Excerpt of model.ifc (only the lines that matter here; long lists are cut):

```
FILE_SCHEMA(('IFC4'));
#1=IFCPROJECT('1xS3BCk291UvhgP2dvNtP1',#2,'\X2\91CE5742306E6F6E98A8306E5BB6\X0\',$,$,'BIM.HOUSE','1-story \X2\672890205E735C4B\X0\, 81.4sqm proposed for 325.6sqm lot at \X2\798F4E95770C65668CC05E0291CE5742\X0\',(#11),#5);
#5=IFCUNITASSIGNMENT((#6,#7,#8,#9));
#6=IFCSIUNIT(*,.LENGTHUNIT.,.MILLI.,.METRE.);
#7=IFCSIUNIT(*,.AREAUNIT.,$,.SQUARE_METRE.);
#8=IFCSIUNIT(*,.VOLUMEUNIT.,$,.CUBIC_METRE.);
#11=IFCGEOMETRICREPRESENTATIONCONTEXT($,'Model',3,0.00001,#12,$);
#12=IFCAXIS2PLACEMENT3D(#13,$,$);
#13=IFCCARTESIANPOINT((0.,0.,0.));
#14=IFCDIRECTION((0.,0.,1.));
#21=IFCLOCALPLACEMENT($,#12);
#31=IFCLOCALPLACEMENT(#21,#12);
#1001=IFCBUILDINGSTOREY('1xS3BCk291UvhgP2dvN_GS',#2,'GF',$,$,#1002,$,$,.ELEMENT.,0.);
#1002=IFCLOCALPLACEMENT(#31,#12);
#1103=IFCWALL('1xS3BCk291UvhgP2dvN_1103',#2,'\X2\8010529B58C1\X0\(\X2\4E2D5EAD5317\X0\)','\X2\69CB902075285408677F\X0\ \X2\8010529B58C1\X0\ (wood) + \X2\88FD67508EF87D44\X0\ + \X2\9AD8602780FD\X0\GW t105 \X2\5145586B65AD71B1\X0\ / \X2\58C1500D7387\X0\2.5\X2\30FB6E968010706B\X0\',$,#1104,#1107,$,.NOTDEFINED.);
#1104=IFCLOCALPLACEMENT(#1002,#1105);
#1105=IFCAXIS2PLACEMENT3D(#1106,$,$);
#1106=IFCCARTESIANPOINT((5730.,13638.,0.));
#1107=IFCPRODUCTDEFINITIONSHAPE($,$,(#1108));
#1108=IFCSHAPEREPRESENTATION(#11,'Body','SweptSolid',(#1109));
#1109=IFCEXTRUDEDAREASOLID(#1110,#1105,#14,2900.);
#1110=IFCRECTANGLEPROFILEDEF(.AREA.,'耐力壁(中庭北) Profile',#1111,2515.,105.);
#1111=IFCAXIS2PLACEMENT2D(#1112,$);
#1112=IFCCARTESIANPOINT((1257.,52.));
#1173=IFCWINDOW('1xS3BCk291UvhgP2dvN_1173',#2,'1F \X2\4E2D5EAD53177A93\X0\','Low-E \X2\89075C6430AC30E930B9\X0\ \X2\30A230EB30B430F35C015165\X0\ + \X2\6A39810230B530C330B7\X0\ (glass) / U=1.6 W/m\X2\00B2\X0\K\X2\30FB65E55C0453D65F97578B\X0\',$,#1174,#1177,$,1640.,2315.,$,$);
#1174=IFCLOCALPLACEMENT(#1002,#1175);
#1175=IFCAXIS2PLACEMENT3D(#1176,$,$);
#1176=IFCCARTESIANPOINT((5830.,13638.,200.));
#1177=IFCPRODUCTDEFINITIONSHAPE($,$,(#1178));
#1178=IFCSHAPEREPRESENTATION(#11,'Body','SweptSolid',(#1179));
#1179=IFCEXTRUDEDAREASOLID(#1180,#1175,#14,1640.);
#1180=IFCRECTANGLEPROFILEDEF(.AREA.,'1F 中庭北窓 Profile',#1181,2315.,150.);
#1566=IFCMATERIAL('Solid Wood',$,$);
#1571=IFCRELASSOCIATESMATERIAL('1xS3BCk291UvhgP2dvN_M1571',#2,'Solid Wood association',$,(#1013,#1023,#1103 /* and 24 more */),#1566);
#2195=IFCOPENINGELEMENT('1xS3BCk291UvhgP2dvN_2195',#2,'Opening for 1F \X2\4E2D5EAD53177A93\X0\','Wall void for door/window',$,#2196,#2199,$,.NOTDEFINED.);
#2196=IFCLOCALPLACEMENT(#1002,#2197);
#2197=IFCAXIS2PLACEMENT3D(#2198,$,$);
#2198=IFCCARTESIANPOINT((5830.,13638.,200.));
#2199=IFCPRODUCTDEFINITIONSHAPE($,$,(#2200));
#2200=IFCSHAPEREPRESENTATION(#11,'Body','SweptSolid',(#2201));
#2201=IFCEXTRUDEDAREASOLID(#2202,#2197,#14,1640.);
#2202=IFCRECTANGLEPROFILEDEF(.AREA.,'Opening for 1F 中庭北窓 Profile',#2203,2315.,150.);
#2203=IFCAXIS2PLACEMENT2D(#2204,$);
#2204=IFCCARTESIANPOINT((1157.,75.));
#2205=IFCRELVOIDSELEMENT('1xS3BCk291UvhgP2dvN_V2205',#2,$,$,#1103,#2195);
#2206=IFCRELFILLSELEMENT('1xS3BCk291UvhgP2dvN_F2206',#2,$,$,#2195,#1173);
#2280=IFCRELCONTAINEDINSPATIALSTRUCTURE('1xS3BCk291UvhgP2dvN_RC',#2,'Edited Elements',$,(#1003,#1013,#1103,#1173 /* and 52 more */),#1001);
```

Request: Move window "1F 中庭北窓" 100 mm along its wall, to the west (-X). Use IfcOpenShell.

```python
import ifcopenshell
import ifcopenshell.api.geometry
import ifcopenshell.util.placement
import ifcopenshell.util.unit

model = ifcopenshell.open("model.ifc")
unit_scale = ifcopenshell.util.unit.calculate_unit_scale(model)

window = model.by_guid("1xS3BCk291UvhgP2dvN_1173")
opening = window.FillsVoids[0].RelatingOpeningElement
wall = opening.VoidsElements[0].RelatingBuildingElement

wall_matrix = ifcopenshell.util.placement.get_local_placement(wall.ObjectPlacement)
shift = wall_matrix[:3, 0] * -0.1 / unit_scale
before = ifcopenshell.util.placement.get_local_placement(window.ObjectPlacement)[:3, 3].copy()

# The window is not placed relative to its opening, so move both.
for product in (opening, window):
    matrix = ifcopenshell.util.placement.get_local_placement(product.ObjectPlacement)
    matrix[:3, 3] += shift
    ifcopenshell.api.geometry.edit_object_placement(model, product=product, matrix=matrix, is_si=False)

after = ifcopenshell.util.placement.get_local_placement(window.ObjectPlacement)[:3, 3]
print("window moved by", (after - before).round(3) + 0.0)

model.write("model_updated.ifc")
```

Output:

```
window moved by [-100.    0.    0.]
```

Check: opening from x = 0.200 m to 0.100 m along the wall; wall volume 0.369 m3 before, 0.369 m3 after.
